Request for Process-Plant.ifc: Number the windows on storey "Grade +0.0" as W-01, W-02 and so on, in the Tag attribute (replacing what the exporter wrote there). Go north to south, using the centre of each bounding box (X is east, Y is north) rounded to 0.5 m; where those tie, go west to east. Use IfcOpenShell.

First a look at what the model holds.

```python
import ifcopenshell
import ifcopenshell.util.element
import ifcopenshell.util.placement

model = ifcopenshell.open("Process-Plant.ifc")
print(model.schema)
storey = next(s for s in model.by_type("IfcBuildingStorey") if s.Name == "Grade +0.0")
windows = [e for e in ifcopenshell.util.element.get_decomposition(storey) if e.is_a("IfcWindow")]
for e in sorted(windows, key=lambda e: e.id()):
    origin = ifcopenshell.util.placement.get_local_placement(e.ObjectPlacement)[:3, 3]
    print(e.id(), e.Tag, e.Name, origin.round(2) + 0.0, sep=" | ")
```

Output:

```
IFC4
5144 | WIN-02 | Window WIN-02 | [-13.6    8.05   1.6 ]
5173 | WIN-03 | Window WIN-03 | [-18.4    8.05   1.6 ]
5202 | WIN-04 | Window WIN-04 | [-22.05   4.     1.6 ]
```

```python
import ifcopenshell
import ifcopenshell.geom
import ifcopenshell.util.element
import ifcopenshell.util.shape

model = ifcopenshell.open("Process-Plant.ifc")
settings = ifcopenshell.geom.settings()
settings.set("use-world-coords", True)


def centre(element):
    shape = ifcopenshell.geom.create_shape(settings, element)
    return ifcopenshell.util.shape.get_bbox_centroid(shape.geometry)


storey = next(s for s in model.by_type("IfcBuildingStorey") if s.Name == "Grade +0.0")
windows = [e for e in ifcopenshell.util.element.get_decomposition(storey) if e.is_a("IfcWindow")]

# Insertion points can sit at a corner or the storey origin, so sort by the geometry (in metres).
centres = {e: centre(e) for e in windows}
windows.sort(key=lambda e: (-round(centres[e][1] / 0.5), centres[e][0]))

for i, e in enumerate(windows, start=1):
    number = f"W-{i:02d}"
    e.Tag = number
    print(e.id(), number)

model.write("Process-Plant_edited.ifc")
```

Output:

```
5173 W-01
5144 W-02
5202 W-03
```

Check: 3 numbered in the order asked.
